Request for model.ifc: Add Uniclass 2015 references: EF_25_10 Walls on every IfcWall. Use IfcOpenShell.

First a look at what the model holds.

```python
import ifcopenshell

model = ifcopenshell.open("model.ifc")
print(model.schema)
print("classifications:", [c.Name for c in model.by_type("IfcClassification")])
for ifc_class in ("IfcDoor", "IfcRoof", "IfcStair", "IfcWall", "IfcWindow"):
    print(ifc_class, len(model.by_type(ifc_class)))
```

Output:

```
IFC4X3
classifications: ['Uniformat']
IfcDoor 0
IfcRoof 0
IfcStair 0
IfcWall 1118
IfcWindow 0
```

```python
import ifcopenshell
import ifcopenshell.api.classification

model = ifcopenshell.open("model.ifc")

system = ifcopenshell.api.classification.add_classification(model, classification="Uniclass 2015")

codes = {
    "IfcWall": ("EF_25_10", "Walls"),
}
for ifc_class, (code, name) in codes.items():
    products = model.by_type(ifc_class)
    ifcopenshell.api.classification.add_reference(
        model, products=products, classification=system, identification=code, name=name
    )
    print(code, len(products))

model.write("model_v2.ifc")
```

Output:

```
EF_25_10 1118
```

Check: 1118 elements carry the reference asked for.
